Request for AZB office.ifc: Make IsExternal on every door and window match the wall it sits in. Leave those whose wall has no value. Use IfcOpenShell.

First a look at what the model holds.

```python
import ifcopenshell
import ifcopenshell.util.element

model = ifcopenshell.open("AZB office.ifc")
print(model.schema)
seen = {}
for e in model.by_type("IfcDoor") + model.by_type("IfcWindow"):
    if not e.FillsVoids:
        continue
    host = e.FillsVoids[0].RelatingOpeningElement.VoidsElements[0].RelatingBuildingElement
    own = ifcopenshell.util.element.get_pset(e, f"Pset_{e.is_a()[3:].removesuffix('StandardCase')}Common", "IsExternal")
    wall = ifcopenshell.util.element.get_pset(host, "Pset_WallCommon", "IsExternal")
    seen[e.is_a(), own, wall] = seen.get((e.is_a(), own, wall), 0) + 1
for (cls, own, wall), count in sorted(seen.items(), key=str):
    print(count, cls, "IsExternal:", own, "| host wall:", wall)
```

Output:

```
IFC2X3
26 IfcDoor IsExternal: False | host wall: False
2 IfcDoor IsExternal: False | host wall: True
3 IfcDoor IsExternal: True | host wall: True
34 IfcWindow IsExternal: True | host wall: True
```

```python
import ifcopenshell
import ifcopenshell.api.pset
import ifcopenshell.util.element

model = ifcopenshell.open("AZB office.ifc")

count = 0
for ifc_class, pset_name in (("IfcDoor", "Pset_DoorCommon"), ("IfcWindow", "Pset_WindowCommon")):
    for e in model.by_type(ifc_class):
        if not e.FillsVoids:
            continue
        host = e.FillsVoids[0].RelatingOpeningElement.VoidsElements[0].RelatingBuildingElement
        external = ifcopenshell.util.element.get_pset(host, "Pset_WallCommon", "IsExternal")
        if external is None or ifcopenshell.util.element.get_pset(e, pset_name, "IsExternal") == external:
            continue
        pset = ifcopenshell.api.pset.add_pset(model, product=e, name=pset_name)
        ifcopenshell.api.pset.edit_pset(model, pset=pset, properties={"IsExternal": external})
        count += 1

print(count, "updated")

model.write("AZB office_rev.ifc")
```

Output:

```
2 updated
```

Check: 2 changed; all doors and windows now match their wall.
